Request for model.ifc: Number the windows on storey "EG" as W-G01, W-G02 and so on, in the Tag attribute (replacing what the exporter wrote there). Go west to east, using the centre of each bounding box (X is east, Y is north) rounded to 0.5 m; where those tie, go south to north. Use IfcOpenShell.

First a look at what the model holds.

```python
import ifcopenshell
import ifcopenshell.util.element
import ifcopenshell.util.placement

model = ifcopenshell.open("model.ifc")
print(model.schema)
storey = next(s for s in model.by_type("IfcBuildingStorey") if s.Name == "EG")
windows = [e for e in ifcopenshell.util.element.get_decomposition(storey) if e.is_a("IfcWindow")]
for e in sorted(windows, key=lambda e: e.id()):
    origin = ifcopenshell.util.placement.get_local_placement(e.ObjectPlacement)[:3, 3]
    print(e.id(), e.Tag, e.Name, origin.round(2) + 0.0, sep=" | ")
```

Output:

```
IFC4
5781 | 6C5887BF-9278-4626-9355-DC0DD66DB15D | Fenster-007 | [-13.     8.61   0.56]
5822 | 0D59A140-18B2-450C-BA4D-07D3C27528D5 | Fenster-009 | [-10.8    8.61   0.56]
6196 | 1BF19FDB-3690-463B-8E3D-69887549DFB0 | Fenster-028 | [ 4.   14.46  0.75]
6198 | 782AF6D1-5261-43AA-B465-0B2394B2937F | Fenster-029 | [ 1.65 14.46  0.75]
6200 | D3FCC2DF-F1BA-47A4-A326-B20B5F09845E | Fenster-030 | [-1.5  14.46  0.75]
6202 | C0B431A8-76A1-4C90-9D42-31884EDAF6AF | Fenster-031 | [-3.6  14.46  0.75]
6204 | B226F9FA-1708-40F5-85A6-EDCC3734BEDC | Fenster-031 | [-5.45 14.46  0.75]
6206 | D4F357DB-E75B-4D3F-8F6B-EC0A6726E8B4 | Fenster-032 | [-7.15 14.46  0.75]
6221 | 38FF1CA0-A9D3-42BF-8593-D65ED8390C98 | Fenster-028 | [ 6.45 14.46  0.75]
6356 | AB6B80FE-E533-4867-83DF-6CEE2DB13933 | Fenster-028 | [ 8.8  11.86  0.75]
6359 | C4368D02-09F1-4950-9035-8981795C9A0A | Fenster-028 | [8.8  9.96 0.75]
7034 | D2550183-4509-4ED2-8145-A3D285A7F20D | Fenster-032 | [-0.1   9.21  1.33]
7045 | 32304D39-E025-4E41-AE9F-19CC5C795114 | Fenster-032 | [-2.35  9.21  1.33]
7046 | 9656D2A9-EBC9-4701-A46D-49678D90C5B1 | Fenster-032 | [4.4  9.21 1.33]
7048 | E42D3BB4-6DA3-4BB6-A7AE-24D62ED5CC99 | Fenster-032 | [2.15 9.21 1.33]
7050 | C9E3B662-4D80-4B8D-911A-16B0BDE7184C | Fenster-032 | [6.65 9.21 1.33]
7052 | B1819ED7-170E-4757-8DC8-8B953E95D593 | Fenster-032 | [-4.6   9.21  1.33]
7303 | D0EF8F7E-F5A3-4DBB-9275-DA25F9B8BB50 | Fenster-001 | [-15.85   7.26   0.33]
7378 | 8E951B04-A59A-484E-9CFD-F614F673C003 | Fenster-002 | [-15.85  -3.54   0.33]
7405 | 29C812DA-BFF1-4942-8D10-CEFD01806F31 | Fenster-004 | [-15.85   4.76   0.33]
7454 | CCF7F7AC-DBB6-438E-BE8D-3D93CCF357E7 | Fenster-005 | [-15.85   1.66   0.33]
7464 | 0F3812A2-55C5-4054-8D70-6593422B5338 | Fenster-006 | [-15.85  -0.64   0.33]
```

```python
import ifcopenshell
import ifcopenshell.geom
import ifcopenshell.util.element
import ifcopenshell.util.shape

model = ifcopenshell.open("model.ifc")
settings = ifcopenshell.geom.settings()
settings.set("use-world-coords", True)


def centre(element):
    shape = ifcopenshell.geom.create_shape(settings, element)
    return ifcopenshell.util.shape.get_bbox_centroid(shape.geometry)


storey = next(s for s in model.by_type("IfcBuildingStorey") if s.Name == "EG")
windows = [e for e in ifcopenshell.util.element.get_decomposition(storey) if e.is_a("IfcWindow")]

# Insertion points can sit at a corner or the storey origin, so sort by the geometry (in metres).
centres = {e: centre(e) for e in windows}
windows.sort(key=lambda e: (round(centres[e][0] / 0.5), centres[e][1]))

for i, e in enumerate(windows, start=1):
    number = f"W-G{i:02d}"
    e.Tag = number
    print(e.id(), number)

model.write("model-out.ifc")
```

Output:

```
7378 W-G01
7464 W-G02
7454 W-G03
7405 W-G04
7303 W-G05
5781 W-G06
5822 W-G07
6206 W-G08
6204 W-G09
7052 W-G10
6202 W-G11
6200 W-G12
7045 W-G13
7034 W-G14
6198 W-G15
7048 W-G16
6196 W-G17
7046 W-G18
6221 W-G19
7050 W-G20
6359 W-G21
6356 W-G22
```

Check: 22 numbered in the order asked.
